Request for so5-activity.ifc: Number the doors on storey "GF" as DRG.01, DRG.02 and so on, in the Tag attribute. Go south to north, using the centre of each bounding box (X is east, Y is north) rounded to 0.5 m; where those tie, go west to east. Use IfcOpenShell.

First a look at what the model holds.

```python
import ifcopenshell
import ifcopenshell.util.element
import ifcopenshell.util.placement

model = ifcopenshell.open("so5-activity.ifc")
print(model.schema)
storey = next(s for s in model.by_type("IfcBuildingStorey") if s.Name == "GF")
doors = [e for e in ifcopenshell.util.element.get_decomposition(storey) if e.is_a("IfcDoor")]
for e in sorted(doors, key=lambda e: e.id()):
    origin = ifcopenshell.util.placement.get_local_placement(e.ObjectPlacement)[:3, 3]
    print(e.id(), e.Tag, e.Name, origin.round(2) + 0.0, sep=" | ")
```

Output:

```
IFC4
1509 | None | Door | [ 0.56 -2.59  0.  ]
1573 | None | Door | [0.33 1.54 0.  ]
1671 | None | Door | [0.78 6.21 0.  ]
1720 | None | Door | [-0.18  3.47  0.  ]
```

```python
import ifcopenshell
import ifcopenshell.geom
import ifcopenshell.util.element
import ifcopenshell.util.shape

model = ifcopenshell.open("so5-activity.ifc")
settings = ifcopenshell.geom.settings()
settings.set("use-world-coords", True)


def centre(element):
    shape = ifcopenshell.geom.create_shape(settings, element)
    return ifcopenshell.util.shape.get_bbox_centroid(shape.geometry)


storey = next(s for s in model.by_type("IfcBuildingStorey") if s.Name == "GF")
doors = [e for e in ifcopenshell.util.element.get_decomposition(storey) if e.is_a("IfcDoor")]

# Insertion points can sit at a corner or the storey origin, so sort by the geometry (in metres).
centres = {e: centre(e) for e in doors}
doors.sort(key=lambda e: (round(centres[e][1] / 0.5), centres[e][0]))

for i, e in enumerate(doors, start=1):
    number = f"DRG.{i:02d}"
    e.Tag = number
    print(e.id(), number)

model.write("so5-activity_rev.ifc")
```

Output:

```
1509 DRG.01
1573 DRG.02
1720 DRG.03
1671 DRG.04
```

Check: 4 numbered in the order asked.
